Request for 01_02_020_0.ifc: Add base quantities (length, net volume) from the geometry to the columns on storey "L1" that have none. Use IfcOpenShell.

First a look at what the model holds.

```python
import ifcopenshell
import ifcopenshell.util.element
import ifcopenshell.util.unit

model = ifcopenshell.open("01_02_020_0.ifc")
print(model.schema)
for unit_type in ("LENGTHUNIT", "AREAUNIT", "VOLUMEUNIT"):
    print(unit_type, ifcopenshell.util.unit.calculate_unit_scale(model, unit_type))
storey = next(s for s in model.by_type("IfcBuildingStorey") if s.Name == "L1")
columns = [e for e in ifcopenshell.util.element.get_decomposition(storey) if e.is_a("IfcColumn")]
for e in sorted(columns, key=lambda e: e.id()):
    print(e.id(), e.is_a(), e.Name, list(ifcopenshell.util.element.get_psets(e, qtos_only=True)), sep=" | ")
```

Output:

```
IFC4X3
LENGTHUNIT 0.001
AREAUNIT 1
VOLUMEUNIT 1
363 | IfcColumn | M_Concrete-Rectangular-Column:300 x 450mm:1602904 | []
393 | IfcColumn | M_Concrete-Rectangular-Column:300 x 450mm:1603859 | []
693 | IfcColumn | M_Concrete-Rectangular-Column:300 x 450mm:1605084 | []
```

```python
import ifcopenshell
import ifcopenshell.api.pset
import ifcopenshell.geom
import ifcopenshell.util.element
import ifcopenshell.util.shape
import ifcopenshell.util.unit

model = ifcopenshell.open("01_02_020_0.ifc")
unit_scale = ifcopenshell.util.unit.calculate_unit_scale(model)
volume_scale = ifcopenshell.util.unit.calculate_unit_scale(model, "VOLUMEUNIT")
settings = ifcopenshell.geom.settings()

storey = next(s for s in model.by_type("IfcBuildingStorey") if s.Name == "L1")
columns = [e for e in ifcopenshell.util.element.get_decomposition(storey) if e.is_a("IfcColumn")]

for e in sorted(columns, key=lambda e: e.id()):
    if ifcopenshell.util.element.get_psets(e, qtos_only=True, should_inherit=False):
        continue
    # Geometry comes back in metres, in the element's own axes.
    shape = ifcopenshell.geom.create_shape(settings, e)
    values = {
        "Length": ifcopenshell.util.shape.get_z(shape.geometry) / unit_scale,
        "NetVolume": ifcopenshell.util.shape.get_volume(shape.geometry) / volume_scale,
    }
    qto = ifcopenshell.api.pset.add_qto(model, product=e, name="Qto_ColumnBaseQuantities")
    ifcopenshell.api.pset.edit_qto(model, qto=qto, properties=values)
    print(e.id(), {k: round(v, 3) for k, v in values.items()})

model.write("01_02_020_0_rev.ifc")
```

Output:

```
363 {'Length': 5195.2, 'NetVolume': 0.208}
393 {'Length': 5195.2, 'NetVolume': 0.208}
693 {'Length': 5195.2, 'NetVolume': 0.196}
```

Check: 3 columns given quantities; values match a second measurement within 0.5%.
